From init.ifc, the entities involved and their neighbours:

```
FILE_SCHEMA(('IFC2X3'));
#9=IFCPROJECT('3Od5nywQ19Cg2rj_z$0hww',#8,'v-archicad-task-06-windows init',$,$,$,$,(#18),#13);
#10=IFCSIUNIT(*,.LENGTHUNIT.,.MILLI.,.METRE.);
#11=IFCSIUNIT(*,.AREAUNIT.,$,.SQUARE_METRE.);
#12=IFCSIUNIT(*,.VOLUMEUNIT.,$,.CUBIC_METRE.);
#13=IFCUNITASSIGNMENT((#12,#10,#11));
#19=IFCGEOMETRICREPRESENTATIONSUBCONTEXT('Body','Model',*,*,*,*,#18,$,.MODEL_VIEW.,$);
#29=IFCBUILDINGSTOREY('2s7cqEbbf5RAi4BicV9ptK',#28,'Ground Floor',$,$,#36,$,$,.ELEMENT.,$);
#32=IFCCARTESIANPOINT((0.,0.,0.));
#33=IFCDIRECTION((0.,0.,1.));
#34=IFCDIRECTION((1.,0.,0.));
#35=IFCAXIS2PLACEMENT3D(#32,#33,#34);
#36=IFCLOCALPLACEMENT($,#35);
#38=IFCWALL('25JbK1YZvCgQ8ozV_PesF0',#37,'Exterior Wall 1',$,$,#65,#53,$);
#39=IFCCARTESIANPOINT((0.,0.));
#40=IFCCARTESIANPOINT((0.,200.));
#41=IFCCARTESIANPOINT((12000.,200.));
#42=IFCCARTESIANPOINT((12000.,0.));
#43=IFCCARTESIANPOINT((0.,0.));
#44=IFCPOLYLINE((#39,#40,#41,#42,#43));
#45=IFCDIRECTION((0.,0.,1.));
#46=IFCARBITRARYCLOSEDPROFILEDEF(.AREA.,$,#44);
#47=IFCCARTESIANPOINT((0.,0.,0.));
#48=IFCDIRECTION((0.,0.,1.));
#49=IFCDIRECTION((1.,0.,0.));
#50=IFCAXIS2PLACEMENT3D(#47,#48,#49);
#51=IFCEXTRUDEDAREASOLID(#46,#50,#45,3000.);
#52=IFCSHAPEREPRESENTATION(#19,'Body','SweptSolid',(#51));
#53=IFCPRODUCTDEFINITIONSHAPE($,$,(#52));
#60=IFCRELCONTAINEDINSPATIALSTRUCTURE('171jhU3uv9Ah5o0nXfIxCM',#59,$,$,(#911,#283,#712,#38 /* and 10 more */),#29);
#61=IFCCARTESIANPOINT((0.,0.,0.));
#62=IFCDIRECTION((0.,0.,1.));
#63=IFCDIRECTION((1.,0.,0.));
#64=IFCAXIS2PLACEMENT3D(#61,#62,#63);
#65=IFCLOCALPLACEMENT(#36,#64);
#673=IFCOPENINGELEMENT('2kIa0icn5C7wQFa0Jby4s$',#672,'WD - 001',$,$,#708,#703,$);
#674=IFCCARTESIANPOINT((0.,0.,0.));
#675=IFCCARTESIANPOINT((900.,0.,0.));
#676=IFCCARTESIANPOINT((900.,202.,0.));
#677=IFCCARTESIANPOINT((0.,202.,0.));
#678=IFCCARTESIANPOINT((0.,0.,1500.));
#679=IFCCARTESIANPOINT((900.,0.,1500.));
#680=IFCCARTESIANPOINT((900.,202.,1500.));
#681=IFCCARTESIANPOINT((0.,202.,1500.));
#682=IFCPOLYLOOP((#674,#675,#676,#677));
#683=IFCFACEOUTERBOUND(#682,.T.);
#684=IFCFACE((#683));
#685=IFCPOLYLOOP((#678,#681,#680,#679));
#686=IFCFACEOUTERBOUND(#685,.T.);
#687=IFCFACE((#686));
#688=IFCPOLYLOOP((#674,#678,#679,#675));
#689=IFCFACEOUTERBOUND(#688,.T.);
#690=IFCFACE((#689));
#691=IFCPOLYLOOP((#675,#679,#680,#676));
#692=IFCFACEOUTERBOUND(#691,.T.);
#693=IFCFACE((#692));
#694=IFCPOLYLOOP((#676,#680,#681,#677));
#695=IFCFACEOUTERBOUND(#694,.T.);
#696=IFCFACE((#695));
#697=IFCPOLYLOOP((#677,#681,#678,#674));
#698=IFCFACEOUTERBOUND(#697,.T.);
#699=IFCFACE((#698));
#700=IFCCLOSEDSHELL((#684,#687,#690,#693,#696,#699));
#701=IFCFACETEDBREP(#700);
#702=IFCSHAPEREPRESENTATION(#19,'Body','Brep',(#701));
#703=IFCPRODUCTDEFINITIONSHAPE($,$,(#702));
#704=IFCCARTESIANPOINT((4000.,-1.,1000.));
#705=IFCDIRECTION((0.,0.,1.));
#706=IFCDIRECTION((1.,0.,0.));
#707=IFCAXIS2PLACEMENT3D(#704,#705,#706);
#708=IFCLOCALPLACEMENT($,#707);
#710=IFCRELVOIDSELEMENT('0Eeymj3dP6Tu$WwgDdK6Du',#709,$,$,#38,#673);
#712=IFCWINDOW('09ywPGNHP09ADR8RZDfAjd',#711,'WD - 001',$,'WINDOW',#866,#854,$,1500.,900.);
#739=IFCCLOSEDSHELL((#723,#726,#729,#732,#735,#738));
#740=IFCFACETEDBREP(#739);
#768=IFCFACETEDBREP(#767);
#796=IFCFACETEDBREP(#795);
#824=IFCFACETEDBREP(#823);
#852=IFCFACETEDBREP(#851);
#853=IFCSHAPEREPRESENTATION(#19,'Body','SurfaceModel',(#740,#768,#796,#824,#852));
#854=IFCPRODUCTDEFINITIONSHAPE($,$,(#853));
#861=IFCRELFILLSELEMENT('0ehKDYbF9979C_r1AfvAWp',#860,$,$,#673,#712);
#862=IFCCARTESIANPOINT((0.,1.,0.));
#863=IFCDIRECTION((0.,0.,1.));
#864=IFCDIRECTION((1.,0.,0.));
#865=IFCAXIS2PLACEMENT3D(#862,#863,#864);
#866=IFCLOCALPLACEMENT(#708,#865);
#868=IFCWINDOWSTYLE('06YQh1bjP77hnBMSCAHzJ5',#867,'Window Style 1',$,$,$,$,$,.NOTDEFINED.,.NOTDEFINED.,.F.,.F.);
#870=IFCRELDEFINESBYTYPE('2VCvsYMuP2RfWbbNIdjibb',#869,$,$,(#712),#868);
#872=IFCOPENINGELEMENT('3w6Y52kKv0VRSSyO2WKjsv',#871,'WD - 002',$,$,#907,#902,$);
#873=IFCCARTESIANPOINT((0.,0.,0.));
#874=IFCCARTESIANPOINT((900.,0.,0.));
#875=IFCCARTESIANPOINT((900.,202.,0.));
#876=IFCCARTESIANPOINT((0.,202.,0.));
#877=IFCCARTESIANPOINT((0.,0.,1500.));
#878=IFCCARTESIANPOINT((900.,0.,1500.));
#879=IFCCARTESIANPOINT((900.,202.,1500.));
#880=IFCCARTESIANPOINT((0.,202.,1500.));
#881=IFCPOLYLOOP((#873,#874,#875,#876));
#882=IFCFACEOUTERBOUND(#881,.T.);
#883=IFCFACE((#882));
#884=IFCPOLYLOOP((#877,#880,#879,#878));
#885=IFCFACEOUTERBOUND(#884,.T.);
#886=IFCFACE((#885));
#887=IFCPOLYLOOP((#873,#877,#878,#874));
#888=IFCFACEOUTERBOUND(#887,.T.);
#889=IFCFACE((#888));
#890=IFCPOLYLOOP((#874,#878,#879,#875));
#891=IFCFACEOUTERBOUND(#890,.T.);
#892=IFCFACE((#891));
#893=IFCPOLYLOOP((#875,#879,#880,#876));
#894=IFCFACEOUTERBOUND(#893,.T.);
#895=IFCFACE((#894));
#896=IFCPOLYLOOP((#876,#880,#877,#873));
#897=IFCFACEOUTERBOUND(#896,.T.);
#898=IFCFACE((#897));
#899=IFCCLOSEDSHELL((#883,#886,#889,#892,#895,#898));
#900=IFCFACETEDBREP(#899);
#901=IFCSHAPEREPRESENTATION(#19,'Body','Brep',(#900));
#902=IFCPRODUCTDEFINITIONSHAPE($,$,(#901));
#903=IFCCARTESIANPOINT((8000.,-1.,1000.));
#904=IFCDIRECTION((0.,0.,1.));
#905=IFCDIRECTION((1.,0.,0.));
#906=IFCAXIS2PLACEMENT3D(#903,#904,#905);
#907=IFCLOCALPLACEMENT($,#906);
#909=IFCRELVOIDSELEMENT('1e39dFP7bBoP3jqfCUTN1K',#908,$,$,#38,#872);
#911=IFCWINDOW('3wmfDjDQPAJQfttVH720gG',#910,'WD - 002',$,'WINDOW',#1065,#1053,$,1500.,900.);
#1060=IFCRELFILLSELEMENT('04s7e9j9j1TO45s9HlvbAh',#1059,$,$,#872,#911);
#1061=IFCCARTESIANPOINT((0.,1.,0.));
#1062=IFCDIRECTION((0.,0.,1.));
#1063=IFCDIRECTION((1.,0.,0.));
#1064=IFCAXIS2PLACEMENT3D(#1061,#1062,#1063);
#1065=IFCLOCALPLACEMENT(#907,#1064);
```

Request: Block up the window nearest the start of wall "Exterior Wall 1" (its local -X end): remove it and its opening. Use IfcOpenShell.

```python
import ifcopenshell
import ifcopenshell.api.feature
import ifcopenshell.api.root
import ifcopenshell.geom
import ifcopenshell.util.shape

model = ifcopenshell.open("init.ifc")
settings = ifcopenshell.geom.settings()


def volume(element):
    """Net volume in cubic metres, openings subtracted."""
    shape = ifcopenshell.geom.create_shape(settings, element)
    return ifcopenshell.util.shape.get_volume(shape.geometry)


window = model.by_id(712)
opening = window.FillsVoids[0].RelatingOpeningElement
wall = opening.VoidsElements[0].RelatingBuildingElement
before = volume(wall)

ifcopenshell.api.root.remove_product(model, product=window)
ifcopenshell.api.feature.remove_feature(model, feature=opening)

after = volume(wall)

print(f"wall volume {before:.3f} -> {after:.3f} m3")

model.write("init_updated.ifc")
```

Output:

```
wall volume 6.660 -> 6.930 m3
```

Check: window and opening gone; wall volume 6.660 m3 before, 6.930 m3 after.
